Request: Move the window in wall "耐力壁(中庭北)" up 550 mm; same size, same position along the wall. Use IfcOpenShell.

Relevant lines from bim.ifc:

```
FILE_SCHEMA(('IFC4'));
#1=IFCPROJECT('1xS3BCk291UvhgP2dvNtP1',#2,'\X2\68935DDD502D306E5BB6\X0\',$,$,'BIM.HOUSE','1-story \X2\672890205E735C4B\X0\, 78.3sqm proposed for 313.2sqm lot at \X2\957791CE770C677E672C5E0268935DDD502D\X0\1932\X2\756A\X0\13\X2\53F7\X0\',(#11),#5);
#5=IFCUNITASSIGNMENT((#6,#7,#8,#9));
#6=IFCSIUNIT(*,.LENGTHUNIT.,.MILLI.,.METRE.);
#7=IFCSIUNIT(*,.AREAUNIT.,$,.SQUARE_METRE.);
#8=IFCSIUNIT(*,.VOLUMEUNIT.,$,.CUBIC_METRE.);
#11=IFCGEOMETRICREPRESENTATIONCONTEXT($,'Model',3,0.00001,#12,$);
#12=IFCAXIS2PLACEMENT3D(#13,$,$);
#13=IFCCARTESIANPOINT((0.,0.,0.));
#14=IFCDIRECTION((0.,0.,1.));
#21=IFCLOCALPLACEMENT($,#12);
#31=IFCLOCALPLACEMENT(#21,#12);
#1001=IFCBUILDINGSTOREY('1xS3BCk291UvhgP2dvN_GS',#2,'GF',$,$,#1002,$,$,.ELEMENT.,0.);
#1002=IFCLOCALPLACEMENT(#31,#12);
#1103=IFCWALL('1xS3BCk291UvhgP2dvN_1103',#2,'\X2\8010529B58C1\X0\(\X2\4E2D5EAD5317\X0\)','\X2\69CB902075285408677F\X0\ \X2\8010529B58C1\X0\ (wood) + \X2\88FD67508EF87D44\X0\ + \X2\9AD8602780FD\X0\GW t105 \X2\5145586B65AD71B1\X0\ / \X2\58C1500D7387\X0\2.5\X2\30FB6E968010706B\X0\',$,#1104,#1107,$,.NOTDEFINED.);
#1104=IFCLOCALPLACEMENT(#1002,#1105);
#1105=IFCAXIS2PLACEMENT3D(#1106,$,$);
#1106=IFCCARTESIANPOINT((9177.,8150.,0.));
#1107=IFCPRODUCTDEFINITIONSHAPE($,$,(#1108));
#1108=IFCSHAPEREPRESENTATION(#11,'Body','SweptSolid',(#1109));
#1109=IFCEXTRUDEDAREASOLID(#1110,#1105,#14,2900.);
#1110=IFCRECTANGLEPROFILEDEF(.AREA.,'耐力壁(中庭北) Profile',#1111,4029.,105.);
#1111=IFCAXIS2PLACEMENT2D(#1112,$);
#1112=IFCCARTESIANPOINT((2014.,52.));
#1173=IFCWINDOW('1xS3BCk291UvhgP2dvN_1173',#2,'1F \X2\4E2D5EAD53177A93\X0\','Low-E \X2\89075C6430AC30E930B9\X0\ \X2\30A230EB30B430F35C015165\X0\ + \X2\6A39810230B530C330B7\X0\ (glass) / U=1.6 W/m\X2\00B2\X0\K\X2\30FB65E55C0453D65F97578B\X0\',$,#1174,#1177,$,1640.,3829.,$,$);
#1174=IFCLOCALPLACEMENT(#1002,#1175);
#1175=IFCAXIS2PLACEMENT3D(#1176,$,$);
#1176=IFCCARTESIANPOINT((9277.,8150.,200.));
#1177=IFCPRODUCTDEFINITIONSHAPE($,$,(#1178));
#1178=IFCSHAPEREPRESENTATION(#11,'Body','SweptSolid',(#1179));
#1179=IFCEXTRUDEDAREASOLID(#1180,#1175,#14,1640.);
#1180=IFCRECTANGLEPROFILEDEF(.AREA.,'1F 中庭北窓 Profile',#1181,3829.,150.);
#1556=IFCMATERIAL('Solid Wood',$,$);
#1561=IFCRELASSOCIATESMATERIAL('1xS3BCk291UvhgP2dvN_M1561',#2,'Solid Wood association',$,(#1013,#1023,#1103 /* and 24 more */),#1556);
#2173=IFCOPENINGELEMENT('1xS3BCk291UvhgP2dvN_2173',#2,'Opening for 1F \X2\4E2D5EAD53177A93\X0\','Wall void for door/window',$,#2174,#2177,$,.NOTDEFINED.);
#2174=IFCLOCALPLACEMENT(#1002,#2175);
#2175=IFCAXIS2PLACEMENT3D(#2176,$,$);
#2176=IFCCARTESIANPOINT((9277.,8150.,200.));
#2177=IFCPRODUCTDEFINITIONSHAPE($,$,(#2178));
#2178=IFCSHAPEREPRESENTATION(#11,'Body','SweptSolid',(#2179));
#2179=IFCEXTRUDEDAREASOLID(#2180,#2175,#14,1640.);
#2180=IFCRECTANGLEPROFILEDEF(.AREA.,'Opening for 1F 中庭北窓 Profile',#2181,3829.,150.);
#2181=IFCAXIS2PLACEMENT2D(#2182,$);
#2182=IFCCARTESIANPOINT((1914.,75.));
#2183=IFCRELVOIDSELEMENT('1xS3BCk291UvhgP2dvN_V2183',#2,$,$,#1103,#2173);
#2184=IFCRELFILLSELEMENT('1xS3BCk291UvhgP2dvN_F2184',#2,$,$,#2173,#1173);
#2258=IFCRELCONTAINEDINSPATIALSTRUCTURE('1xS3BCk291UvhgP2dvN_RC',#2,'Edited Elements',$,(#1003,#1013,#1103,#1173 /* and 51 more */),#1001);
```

```python
import numpy as np
import ifcopenshell
import ifcopenshell.api.geometry
import ifcopenshell.util.placement
import ifcopenshell.util.unit

model = ifcopenshell.open("bim.ifc")
unit_scale = ifcopenshell.util.unit.calculate_unit_scale(model)

window = model.by_guid("1xS3BCk291UvhgP2dvN_1173")
opening = window.FillsVoids[0].RelatingOpeningElement
dz = 0.55 / unit_scale

shift = np.array([0.0, 0.0, dz])
# The window is not placed relative to its opening, so move both.
for product in (opening, window):
    matrix = ifcopenshell.util.placement.get_local_placement(product.ObjectPlacement)
    matrix[:3, 3] += shift
    ifcopenshell.api.geometry.edit_object_placement(model, product=product, matrix=matrix, is_si=False)

print(f"moved by {dz * unit_scale:+.3f} m")

model.write("bim_v2.ifc")
```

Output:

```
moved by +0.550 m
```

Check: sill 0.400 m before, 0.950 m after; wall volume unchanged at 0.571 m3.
